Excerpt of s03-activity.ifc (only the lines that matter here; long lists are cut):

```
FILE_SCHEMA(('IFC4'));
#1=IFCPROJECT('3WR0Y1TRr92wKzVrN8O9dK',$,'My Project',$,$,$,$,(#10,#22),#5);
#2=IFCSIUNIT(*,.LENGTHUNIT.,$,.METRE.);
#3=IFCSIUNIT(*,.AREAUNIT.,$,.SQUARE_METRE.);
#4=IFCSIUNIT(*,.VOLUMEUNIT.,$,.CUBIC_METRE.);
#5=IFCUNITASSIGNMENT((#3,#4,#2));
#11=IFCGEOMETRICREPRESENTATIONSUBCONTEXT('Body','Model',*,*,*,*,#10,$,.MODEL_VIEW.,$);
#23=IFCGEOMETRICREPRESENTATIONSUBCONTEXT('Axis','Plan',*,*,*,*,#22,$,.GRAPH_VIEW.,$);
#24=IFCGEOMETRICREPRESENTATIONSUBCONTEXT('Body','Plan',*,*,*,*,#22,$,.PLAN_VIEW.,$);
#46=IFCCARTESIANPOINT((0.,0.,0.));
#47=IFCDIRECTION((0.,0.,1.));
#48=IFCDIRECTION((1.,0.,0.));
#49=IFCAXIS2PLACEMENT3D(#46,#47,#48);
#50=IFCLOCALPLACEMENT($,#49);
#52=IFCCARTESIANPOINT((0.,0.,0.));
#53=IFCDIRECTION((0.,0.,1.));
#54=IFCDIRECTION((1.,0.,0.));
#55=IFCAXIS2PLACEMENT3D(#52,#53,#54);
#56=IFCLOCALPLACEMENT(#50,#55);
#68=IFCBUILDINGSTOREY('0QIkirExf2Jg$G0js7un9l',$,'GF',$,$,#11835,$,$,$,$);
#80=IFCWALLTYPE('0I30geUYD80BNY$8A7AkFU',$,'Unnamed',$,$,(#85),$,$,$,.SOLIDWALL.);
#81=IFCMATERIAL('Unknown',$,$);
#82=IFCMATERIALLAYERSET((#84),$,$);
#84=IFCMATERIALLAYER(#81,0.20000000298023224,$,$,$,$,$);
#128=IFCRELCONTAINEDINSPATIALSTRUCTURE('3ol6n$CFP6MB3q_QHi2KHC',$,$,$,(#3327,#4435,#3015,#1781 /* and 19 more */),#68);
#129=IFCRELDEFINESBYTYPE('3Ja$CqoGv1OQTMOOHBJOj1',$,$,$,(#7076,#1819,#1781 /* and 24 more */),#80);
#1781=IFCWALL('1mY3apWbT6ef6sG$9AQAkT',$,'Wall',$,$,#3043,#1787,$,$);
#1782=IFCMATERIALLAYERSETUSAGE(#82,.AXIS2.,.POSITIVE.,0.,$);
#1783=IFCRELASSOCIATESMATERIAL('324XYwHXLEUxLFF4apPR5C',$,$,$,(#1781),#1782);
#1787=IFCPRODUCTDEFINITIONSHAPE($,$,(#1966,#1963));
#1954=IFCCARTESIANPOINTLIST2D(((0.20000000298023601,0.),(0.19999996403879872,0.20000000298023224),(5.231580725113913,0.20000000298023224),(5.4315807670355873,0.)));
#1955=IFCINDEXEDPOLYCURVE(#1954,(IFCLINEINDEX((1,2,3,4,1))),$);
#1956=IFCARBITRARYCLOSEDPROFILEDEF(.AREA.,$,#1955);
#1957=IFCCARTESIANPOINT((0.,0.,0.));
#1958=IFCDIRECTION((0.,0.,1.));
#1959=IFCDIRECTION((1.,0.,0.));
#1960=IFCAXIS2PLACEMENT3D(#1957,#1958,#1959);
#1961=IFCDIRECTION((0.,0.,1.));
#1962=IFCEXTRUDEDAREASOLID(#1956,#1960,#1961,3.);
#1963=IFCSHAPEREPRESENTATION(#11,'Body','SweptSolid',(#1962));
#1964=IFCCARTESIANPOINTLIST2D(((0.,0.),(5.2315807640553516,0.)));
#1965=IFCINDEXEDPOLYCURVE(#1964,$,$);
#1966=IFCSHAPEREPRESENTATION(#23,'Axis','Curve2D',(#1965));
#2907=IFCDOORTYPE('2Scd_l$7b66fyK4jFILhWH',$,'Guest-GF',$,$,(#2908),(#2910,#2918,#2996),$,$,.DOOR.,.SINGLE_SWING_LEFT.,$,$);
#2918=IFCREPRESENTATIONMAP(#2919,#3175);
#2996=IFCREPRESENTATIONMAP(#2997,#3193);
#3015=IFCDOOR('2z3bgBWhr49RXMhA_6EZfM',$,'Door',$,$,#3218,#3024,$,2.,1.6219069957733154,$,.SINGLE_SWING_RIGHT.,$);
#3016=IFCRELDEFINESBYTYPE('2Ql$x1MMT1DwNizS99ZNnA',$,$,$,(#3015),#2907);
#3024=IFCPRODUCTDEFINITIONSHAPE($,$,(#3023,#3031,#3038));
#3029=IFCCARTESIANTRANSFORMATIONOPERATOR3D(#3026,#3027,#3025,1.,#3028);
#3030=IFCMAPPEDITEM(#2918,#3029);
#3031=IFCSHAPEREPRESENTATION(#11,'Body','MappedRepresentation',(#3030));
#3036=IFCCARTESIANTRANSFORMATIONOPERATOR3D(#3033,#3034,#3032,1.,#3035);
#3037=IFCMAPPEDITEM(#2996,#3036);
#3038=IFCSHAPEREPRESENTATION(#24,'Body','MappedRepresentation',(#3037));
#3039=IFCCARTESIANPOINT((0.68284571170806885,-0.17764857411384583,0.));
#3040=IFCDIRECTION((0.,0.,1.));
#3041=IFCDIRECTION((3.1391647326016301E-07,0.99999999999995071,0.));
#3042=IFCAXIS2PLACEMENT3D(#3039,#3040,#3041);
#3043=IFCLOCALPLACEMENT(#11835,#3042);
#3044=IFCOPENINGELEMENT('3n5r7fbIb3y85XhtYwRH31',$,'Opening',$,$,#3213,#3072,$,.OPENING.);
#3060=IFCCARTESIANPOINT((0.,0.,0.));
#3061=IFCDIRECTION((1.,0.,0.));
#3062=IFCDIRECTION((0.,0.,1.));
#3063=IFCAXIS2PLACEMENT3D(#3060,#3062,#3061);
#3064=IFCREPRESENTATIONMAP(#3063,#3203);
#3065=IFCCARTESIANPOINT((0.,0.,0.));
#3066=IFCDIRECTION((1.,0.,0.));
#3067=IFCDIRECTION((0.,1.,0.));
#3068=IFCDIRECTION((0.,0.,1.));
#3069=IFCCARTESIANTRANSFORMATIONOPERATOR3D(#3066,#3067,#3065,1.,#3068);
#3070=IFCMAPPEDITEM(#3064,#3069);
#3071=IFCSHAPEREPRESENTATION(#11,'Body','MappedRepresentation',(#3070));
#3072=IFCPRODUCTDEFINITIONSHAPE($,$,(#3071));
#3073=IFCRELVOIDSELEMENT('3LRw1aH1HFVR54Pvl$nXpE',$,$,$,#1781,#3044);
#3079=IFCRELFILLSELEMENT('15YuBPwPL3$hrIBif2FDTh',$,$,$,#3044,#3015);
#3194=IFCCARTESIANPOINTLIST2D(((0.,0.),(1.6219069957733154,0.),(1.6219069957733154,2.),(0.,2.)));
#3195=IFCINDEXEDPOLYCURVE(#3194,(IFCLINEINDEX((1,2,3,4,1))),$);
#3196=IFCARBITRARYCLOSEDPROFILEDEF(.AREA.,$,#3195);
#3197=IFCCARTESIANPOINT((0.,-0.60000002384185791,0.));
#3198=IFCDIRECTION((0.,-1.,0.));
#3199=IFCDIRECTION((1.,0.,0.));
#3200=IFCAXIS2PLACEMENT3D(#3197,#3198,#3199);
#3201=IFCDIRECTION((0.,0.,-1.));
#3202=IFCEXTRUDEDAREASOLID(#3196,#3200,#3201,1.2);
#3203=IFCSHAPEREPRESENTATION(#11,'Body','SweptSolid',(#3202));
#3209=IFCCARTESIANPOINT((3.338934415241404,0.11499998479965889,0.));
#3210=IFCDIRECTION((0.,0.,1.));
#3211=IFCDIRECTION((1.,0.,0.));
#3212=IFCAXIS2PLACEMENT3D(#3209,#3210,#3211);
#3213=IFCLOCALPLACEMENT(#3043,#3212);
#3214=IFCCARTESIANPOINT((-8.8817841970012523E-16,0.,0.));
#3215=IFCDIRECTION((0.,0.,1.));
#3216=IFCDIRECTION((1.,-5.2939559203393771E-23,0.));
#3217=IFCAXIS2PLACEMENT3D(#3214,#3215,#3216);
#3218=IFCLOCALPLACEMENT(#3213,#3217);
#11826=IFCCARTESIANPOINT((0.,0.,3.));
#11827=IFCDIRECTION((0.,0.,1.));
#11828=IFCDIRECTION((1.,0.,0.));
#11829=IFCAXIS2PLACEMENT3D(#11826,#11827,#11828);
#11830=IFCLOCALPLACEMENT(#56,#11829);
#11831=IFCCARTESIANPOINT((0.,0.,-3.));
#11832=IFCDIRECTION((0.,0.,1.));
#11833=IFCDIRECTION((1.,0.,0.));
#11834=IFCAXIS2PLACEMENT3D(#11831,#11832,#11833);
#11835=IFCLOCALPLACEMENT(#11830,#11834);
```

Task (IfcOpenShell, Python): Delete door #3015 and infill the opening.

```python
import ifcopenshell
import ifcopenshell.api.feature
import ifcopenshell.api.root
import ifcopenshell.geom
import ifcopenshell.util.shape

model = ifcopenshell.open("s03-activity.ifc")
settings = ifcopenshell.geom.settings()


def volume(element):
    """Net volume in cubic metres, openings subtracted."""
    shape = ifcopenshell.geom.create_shape(settings, element)
    return ifcopenshell.util.shape.get_volume(shape.geometry)


door = model.by_id(3015)
opening = door.FillsVoids[0].RelatingOpeningElement
wall = opening.VoidsElements[0].RelatingBuildingElement
before = volume(wall)

ifcopenshell.api.root.remove_product(model, product=door)
ifcopenshell.api.feature.remove_feature(model, feature=opening)

after = volume(wall)

print(f"wall volume {before:.3f} -> {after:.3f} m3")

model.write("s03-activity_rev.ifc")
```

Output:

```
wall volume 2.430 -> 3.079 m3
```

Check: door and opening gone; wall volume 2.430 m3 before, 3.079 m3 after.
